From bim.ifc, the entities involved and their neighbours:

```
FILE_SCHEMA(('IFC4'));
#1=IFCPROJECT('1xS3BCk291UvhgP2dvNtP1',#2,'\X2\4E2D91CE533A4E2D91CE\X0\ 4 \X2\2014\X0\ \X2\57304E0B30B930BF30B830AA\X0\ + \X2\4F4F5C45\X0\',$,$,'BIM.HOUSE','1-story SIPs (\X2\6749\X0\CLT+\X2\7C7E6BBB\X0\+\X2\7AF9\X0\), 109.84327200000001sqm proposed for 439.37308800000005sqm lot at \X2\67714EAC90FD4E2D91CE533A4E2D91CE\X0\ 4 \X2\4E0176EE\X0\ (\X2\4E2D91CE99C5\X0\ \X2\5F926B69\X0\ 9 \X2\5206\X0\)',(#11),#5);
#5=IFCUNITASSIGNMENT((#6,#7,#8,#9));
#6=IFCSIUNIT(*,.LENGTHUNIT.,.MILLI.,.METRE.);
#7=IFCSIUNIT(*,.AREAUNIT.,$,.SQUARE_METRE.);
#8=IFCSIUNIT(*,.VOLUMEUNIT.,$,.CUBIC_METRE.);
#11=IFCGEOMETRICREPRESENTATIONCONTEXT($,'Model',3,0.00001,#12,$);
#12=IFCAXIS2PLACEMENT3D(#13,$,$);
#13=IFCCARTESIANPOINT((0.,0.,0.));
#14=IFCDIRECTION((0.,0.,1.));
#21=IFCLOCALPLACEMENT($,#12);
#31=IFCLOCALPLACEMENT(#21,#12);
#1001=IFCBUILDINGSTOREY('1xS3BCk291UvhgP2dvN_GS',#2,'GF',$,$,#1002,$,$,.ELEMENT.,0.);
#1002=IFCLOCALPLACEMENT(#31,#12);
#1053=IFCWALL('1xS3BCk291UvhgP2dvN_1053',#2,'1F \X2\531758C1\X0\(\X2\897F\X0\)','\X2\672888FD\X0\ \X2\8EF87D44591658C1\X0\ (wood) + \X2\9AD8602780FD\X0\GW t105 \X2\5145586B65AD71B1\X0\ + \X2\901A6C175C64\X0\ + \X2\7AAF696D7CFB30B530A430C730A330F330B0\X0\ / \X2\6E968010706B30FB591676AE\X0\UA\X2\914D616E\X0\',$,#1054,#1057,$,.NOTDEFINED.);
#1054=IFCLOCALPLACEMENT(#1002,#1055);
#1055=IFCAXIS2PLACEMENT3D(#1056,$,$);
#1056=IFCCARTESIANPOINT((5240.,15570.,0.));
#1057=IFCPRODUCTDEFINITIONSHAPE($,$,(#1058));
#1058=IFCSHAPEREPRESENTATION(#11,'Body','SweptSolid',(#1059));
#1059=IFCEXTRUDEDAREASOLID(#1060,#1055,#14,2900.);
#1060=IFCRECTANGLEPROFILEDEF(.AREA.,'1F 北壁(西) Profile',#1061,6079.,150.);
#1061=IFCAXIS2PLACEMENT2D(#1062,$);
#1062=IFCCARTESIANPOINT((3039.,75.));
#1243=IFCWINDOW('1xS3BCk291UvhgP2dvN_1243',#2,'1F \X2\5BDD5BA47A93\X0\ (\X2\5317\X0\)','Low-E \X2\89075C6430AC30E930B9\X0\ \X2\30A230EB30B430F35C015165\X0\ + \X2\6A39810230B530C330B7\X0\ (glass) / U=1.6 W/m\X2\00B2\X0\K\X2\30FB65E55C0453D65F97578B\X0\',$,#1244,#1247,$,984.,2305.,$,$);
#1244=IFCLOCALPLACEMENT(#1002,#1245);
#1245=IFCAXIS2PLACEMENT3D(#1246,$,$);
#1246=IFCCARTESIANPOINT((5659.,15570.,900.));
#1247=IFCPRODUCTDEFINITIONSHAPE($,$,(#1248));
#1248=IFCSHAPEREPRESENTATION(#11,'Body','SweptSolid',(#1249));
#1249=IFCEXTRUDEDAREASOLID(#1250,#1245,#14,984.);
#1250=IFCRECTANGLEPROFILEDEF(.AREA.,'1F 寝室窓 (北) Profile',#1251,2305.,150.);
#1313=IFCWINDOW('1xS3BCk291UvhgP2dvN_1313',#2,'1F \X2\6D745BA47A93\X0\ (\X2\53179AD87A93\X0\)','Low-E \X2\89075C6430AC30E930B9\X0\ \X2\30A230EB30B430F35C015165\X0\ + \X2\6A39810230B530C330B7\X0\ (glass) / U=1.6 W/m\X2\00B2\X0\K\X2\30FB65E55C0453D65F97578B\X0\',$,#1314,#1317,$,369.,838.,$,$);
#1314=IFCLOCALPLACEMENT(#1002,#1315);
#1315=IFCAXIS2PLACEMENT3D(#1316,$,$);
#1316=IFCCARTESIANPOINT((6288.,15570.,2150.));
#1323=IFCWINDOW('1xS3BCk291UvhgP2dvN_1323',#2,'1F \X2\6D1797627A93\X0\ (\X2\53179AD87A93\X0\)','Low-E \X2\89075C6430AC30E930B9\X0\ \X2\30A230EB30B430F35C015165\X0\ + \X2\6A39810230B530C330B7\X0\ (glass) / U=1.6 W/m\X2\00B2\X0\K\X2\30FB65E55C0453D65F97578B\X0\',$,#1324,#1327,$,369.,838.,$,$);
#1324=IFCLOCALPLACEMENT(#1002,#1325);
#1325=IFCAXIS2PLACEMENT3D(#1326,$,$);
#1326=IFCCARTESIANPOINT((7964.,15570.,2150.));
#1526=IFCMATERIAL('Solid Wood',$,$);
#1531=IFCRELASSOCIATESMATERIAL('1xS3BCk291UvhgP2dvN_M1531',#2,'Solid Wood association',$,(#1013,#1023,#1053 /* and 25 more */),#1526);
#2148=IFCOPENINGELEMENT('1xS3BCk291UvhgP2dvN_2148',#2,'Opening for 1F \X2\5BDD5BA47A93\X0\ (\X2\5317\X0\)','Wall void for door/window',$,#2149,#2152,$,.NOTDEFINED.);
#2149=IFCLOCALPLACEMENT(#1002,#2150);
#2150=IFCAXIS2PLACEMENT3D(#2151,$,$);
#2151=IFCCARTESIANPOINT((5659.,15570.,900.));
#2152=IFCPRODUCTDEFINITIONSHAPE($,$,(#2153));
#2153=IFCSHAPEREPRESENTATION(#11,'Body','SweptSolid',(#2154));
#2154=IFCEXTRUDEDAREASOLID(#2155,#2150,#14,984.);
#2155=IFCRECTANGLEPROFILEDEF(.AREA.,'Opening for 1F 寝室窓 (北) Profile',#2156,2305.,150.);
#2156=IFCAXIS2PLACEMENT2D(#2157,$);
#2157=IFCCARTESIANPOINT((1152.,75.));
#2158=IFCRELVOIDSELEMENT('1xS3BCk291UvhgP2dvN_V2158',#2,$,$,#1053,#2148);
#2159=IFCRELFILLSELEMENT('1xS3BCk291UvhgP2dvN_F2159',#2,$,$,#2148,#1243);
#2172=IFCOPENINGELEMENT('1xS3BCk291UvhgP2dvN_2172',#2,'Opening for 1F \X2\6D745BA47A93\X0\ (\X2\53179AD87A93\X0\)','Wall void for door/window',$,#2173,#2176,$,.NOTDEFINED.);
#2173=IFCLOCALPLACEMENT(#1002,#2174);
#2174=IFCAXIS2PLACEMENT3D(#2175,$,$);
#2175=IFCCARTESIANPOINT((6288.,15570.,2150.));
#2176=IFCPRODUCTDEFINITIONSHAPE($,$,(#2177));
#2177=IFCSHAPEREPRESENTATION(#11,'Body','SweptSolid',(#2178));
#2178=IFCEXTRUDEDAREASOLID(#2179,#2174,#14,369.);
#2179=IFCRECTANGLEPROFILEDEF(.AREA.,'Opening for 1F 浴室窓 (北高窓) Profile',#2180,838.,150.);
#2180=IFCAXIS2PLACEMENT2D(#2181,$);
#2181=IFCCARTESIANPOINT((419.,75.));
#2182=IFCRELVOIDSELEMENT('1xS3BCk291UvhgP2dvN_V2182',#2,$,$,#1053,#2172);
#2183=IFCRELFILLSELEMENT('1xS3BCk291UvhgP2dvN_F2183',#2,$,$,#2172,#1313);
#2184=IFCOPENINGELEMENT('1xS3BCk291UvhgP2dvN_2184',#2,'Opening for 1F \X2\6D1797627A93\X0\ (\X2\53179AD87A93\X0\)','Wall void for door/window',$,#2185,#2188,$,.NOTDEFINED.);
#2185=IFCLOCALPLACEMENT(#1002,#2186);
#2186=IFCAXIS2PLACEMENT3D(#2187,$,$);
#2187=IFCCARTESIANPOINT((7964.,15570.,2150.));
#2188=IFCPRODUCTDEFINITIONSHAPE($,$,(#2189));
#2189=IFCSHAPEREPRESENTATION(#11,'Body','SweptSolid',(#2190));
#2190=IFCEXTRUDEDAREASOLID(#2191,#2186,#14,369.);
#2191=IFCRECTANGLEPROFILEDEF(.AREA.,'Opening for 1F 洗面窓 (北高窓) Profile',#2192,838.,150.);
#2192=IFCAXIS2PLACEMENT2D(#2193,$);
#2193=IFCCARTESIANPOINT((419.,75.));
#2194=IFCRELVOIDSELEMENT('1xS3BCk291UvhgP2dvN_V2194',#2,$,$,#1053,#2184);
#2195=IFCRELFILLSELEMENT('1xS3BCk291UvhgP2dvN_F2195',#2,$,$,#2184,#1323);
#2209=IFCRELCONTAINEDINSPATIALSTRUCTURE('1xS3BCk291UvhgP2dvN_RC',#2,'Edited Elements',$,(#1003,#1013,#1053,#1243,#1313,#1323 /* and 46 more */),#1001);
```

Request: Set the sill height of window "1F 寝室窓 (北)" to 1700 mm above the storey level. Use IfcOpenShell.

```python
import numpy as np
import ifcopenshell
import ifcopenshell.api.geometry
import ifcopenshell.geom
import ifcopenshell.util.element
import ifcopenshell.util.placement
import ifcopenshell.util.shape
import ifcopenshell.util.unit

model = ifcopenshell.open("bim.ifc")
unit_scale = ifcopenshell.util.unit.calculate_unit_scale(model)

window = model.by_guid("1xS3BCk291UvhgP2dvN_1243")
opening = window.FillsVoids[0].RelatingOpeningElement
storey = ifcopenshell.util.element.get_container(window, ifc_class="IfcBuildingStorey")
level = ifcopenshell.util.placement.get_local_placement(storey.ObjectPlacement)[2, 3]

# The opening's origin need not be at the sill, so measure its lowest point.
shape = ifcopenshell.geom.create_shape(ifcopenshell.geom.settings(), opening)
bottom = ifcopenshell.util.shape.get_shape_bottom_elevation(shape, shape.geometry) / unit_scale
dz = level + 1700.0 - bottom

shift = np.array([0.0, 0.0, dz])
# The window is not placed relative to its opening, so move both.
for product in (opening, window):
    matrix = ifcopenshell.util.placement.get_local_placement(product.ObjectPlacement)
    matrix[:3, 3] += shift
    ifcopenshell.api.geometry.edit_object_placement(model, product=product, matrix=matrix, is_si=False)

print(f"moved by {dz * unit_scale:+.3f} m")

model.write("bim_v2.ifc")
```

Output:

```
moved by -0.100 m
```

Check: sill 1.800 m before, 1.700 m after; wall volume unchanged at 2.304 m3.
